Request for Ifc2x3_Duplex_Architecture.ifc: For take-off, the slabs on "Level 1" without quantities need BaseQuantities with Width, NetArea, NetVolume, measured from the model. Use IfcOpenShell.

First a look at what the model holds.

```python
import ifcopenshell
import ifcopenshell.util.element
import ifcopenshell.util.unit

model = ifcopenshell.open("Ifc2x3_Duplex_Architecture.ifc")
print(model.schema)
for unit_type in ("LENGTHUNIT", "AREAUNIT", "VOLUMEUNIT"):
    print(unit_type, ifcopenshell.util.unit.calculate_unit_scale(model, unit_type))
storey = next(s for s in model.by_type("IfcBuildingStorey") if s.Name == "Level 1")
slabs = [e for e in ifcopenshell.util.element.get_decomposition(storey) if e.is_a("IfcSlab")]
for e in sorted(slabs, key=lambda e: e.id()):
    print(e.id(), e.is_a(), e.Name, list(ifcopenshell.util.element.get_psets(e, qtos_only=True)), sep=" | ")
```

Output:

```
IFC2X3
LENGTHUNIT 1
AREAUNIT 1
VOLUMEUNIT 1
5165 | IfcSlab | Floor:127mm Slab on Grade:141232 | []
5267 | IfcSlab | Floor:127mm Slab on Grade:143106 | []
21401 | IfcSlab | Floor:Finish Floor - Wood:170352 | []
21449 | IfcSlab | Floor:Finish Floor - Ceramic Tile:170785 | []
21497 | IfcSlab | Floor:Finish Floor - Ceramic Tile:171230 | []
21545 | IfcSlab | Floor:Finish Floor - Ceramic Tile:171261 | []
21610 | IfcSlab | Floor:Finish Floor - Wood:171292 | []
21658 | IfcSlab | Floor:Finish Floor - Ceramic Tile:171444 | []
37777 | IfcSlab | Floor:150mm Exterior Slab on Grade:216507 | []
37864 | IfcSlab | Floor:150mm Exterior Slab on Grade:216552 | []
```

```python
import ifcopenshell
import ifcopenshell.api.pset
import ifcopenshell.geom
import ifcopenshell.util.element
import ifcopenshell.util.shape
import ifcopenshell.util.unit

model = ifcopenshell.open("Ifc2x3_Duplex_Architecture.ifc")
unit_scale = ifcopenshell.util.unit.calculate_unit_scale(model)
area_scale = ifcopenshell.util.unit.calculate_unit_scale(model, "AREAUNIT")
volume_scale = ifcopenshell.util.unit.calculate_unit_scale(model, "VOLUMEUNIT")
settings = ifcopenshell.geom.settings()

storey = next(s for s in model.by_type("IfcBuildingStorey") if s.Name == "Level 1")
slabs = [e for e in ifcopenshell.util.element.get_decomposition(storey) if e.is_a("IfcSlab")]

for e in sorted(slabs, key=lambda e: e.id()):
    if ifcopenshell.util.element.get_psets(e, qtos_only=True, should_inherit=False):
        continue
    # Geometry comes back in metres, in the element's own axes.
    shape = ifcopenshell.geom.create_shape(settings, e)
    values = {
        "Width": ifcopenshell.util.shape.get_z(shape.geometry) / unit_scale,
        "NetArea": ifcopenshell.util.shape.get_footprint_area(shape.geometry) / area_scale,
        "NetVolume": ifcopenshell.util.shape.get_volume(shape.geometry) / volume_scale,
    }
    qto = ifcopenshell.api.pset.add_qto(model, product=e, name="BaseQuantities")
    ifcopenshell.api.pset.edit_qto(model, qto=qto, properties=values)
    print(e.id(), {k: round(v, 3) for k, v in values.items()})

model.write("Ifc2x3_Duplex_Architecture_v2.ifc")
```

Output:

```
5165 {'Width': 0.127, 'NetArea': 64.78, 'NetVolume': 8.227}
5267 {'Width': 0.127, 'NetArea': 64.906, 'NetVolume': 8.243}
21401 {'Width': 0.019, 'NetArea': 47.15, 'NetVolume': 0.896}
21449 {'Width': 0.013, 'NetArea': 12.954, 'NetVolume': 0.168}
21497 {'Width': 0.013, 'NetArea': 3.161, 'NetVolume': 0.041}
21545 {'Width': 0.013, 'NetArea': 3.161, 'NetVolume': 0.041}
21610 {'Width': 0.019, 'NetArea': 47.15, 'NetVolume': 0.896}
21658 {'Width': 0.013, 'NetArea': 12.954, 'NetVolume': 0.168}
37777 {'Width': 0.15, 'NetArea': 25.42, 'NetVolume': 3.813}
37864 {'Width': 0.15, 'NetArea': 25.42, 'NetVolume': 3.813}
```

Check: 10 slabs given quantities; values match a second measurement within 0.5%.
